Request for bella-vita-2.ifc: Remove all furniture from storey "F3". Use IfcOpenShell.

First a look at what the model holds.

```python
import ifcopenshell
import ifcopenshell.util.element

model = ifcopenshell.open("bella-vita-2.ifc")
print(model.schema)
storey = next(s for s in model.by_type("IfcBuildingStorey") if s.Name == "F3")
furniture = [e for e in ifcopenshell.util.element.get_decomposition(storey) if e.is_a("IfcFurnishingElement")]
seen = {}
for e in furniture:
    element_type = ifcopenshell.util.element.get_type(e)
    name = element_type.Name if element_type not in (None, e) else None
    seen[name] = seen.get(name, 0) + 1
for name, count in sorted(seen.items(), key=str):
    print(count, "x", name)
```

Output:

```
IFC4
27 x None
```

```python
import ifcopenshell
import ifcopenshell.api.root
import ifcopenshell.util.element

model = ifcopenshell.open("bella-vita-2.ifc")

storey = next(s for s in model.by_type("IfcBuildingStorey") if s.Name == "F3")
furniture = [e for e in ifcopenshell.util.element.get_decomposition(storey) if e.is_a("IfcFurnishingElement")]

for e in furniture:
    ifcopenshell.api.root.remove_product(model, product=e)
print(len(furniture), "removed")

model.write("bella-vita-2-out.ifc")
```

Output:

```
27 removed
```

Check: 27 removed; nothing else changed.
